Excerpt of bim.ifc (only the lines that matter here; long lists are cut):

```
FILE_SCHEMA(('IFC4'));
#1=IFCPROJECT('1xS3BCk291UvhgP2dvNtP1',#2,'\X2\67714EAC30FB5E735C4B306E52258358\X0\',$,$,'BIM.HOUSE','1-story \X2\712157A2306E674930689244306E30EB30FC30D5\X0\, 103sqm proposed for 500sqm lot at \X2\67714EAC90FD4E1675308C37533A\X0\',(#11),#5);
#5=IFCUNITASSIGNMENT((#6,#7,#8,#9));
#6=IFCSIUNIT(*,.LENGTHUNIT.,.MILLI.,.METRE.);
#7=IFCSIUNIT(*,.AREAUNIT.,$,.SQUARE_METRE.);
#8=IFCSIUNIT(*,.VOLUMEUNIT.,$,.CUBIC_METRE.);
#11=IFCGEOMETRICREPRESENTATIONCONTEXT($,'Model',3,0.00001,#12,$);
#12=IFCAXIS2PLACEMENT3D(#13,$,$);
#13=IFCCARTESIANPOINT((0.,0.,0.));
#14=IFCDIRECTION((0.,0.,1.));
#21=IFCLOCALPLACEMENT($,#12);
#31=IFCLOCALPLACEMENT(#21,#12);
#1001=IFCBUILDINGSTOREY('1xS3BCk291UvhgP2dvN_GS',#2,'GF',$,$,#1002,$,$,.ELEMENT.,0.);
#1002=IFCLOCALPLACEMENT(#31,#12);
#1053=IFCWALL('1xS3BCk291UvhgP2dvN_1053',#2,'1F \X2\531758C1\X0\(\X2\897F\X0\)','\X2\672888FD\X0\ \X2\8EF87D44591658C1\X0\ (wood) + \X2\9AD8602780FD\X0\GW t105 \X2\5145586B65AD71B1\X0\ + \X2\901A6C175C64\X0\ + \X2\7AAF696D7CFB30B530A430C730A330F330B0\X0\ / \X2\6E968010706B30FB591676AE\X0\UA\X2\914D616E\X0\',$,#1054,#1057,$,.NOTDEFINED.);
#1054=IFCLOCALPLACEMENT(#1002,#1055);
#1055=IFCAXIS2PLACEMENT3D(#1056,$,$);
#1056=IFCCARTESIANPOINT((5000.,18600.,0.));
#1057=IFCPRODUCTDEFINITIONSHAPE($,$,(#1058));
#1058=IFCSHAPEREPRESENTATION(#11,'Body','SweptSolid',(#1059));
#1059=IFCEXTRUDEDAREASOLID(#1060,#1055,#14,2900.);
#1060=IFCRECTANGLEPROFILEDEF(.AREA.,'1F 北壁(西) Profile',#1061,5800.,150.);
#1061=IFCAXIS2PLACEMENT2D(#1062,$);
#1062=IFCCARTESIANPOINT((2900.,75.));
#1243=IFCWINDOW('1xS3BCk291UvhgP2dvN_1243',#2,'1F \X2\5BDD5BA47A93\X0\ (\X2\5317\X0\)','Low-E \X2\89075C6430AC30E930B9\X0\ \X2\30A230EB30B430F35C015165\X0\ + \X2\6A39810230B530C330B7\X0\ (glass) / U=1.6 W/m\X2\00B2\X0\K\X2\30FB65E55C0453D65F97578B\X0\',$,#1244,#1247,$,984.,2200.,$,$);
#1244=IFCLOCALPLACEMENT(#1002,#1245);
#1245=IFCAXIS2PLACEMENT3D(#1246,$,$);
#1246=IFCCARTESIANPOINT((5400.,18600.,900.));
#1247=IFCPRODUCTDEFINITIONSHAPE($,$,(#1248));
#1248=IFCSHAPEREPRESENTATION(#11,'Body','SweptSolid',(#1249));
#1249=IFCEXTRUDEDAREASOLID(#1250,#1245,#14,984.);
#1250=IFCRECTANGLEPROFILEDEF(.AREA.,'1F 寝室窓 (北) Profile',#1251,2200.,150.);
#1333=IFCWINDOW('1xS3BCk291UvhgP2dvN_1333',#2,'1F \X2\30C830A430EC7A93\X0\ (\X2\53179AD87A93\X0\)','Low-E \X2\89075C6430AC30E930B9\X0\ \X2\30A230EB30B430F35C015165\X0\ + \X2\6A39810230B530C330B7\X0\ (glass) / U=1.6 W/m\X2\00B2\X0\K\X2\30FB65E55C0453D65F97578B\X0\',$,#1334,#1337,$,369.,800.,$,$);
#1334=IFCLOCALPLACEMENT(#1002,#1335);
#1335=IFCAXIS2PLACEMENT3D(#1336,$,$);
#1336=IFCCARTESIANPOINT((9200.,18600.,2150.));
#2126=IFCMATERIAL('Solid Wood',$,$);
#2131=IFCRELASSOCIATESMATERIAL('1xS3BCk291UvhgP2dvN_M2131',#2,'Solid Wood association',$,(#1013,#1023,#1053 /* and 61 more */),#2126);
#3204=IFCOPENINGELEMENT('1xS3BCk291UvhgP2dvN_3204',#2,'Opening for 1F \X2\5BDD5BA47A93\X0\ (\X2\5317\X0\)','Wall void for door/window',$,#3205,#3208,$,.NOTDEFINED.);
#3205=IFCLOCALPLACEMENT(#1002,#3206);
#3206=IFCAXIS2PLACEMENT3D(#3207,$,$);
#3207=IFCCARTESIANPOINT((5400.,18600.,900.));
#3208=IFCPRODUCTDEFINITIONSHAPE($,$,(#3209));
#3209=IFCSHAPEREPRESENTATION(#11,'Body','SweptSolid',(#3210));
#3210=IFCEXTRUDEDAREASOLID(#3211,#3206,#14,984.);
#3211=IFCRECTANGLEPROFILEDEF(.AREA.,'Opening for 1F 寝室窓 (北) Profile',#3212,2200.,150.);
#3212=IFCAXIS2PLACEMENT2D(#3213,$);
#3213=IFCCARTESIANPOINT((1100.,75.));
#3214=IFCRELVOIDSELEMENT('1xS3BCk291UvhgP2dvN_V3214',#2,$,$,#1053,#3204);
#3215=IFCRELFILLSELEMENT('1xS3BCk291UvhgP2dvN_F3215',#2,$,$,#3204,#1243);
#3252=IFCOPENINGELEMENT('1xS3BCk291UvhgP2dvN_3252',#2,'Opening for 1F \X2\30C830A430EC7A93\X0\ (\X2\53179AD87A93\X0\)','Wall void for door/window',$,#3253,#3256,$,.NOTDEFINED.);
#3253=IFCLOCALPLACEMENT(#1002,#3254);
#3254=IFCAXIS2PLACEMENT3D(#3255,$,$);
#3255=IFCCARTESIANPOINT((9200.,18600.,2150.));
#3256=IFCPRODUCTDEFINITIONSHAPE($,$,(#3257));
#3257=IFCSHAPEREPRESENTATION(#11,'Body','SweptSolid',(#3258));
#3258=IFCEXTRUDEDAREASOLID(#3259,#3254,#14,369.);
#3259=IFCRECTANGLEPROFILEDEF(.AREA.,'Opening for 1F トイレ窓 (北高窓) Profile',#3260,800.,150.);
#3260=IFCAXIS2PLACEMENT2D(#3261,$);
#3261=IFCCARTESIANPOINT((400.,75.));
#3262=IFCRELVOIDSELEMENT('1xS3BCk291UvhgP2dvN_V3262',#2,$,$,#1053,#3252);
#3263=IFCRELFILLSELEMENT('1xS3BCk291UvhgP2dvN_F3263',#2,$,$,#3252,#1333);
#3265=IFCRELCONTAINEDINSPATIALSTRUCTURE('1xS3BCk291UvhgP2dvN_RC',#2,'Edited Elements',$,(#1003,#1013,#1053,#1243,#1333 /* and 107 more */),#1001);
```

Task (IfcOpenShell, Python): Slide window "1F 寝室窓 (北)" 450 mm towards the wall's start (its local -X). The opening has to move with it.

```python
import ifcopenshell
import ifcopenshell.api.geometry
import ifcopenshell.util.placement

model = ifcopenshell.open("bim.ifc")

window = model.by_guid("1xS3BCk291UvhgP2dvN_1243")
opening = window.FillsVoids[0].RelatingOpeningElement
wall = opening.VoidsElements[0].RelatingBuildingElement

wall_matrix = ifcopenshell.util.placement.get_local_placement(wall.ObjectPlacement)
shift = wall_matrix[:3, 0] * -450.0
before = ifcopenshell.util.placement.get_local_placement(window.ObjectPlacement)[:3, 3].copy()

# The window is not placed relative to its opening, so move both.
for product in (opening, window):
    matrix = ifcopenshell.util.placement.get_local_placement(product.ObjectPlacement)
    matrix[:3, 3] += shift
    ifcopenshell.api.geometry.edit_object_placement(model, product=product, matrix=matrix, is_si=False)

after = ifcopenshell.util.placement.get_local_placement(window.ObjectPlacement)[:3, 3]
print("window moved by", (after - before).round(3) + 0.0)

model.write("bim-out.ifc")
```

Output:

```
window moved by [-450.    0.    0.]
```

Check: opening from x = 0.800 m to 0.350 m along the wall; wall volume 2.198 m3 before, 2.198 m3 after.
